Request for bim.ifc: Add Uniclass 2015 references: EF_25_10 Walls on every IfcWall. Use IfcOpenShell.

First a look at what the model holds.

```python
import ifcopenshell

model = ifcopenshell.open("bim.ifc")
print(model.schema)
print("classifications:", [c.Name for c in model.by_type("IfcClassification")])
for ifc_class in ("IfcDoor", "IfcRoof", "IfcStair", "IfcWall", "IfcWindow"):
    print(ifc_class, len(model.by_type(ifc_class)))
```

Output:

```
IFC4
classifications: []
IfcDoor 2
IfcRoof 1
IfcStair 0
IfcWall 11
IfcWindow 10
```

```python
import ifcopenshell
import ifcopenshell.api.classification

model = ifcopenshell.open("bim.ifc")

system = ifcopenshell.api.classification.add_classification(model, classification="Uniclass 2015")

codes = {
    "IfcWall": ("EF_25_10", "Walls"),
}
for ifc_class, (code, name) in codes.items():
    products = model.by_type(ifc_class)
    ifcopenshell.api.classification.add_reference(
        model, products=products, classification=system, identification=code, name=name
    )
    print(code, len(products))

model.write("bim-out.ifc")
```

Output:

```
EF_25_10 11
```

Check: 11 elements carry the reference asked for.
